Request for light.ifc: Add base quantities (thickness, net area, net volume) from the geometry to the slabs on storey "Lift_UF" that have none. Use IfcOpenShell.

First a look at what the model holds.

```python
import ifcopenshell
import ifcopenshell.util.element
import ifcopenshell.util.unit

model = ifcopenshell.open("light.ifc")
print(model.schema)
for unit_type in ("LENGTHUNIT", "AREAUNIT", "VOLUMEUNIT"):
    print(unit_type, ifcopenshell.util.unit.calculate_unit_scale(model, unit_type))
storey = next(s for s in model.by_type("IfcBuildingStorey") if s.Name == "Lift_UF")
slabs = [e for e in ifcopenshell.util.element.get_decomposition(storey) if e.is_a("IfcSlab")]
for e in sorted(slabs, key=lambda e: e.id()):
    print(e.id(), e.is_a(), e.Name, list(ifcopenshell.util.element.get_psets(e, qtos_only=True)), sep=" | ")
```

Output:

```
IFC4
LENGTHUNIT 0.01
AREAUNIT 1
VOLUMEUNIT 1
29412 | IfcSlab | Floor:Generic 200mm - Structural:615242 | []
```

```python
import ifcopenshell
import ifcopenshell.api.pset
import ifcopenshell.geom
import ifcopenshell.util.element
import ifcopenshell.util.shape
import ifcopenshell.util.unit

model = ifcopenshell.open("light.ifc")
unit_scale = ifcopenshell.util.unit.calculate_unit_scale(model)
area_scale = ifcopenshell.util.unit.calculate_unit_scale(model, "AREAUNIT")
volume_scale = ifcopenshell.util.unit.calculate_unit_scale(model, "VOLUMEUNIT")
settings = ifcopenshell.geom.settings()

storey = next(s for s in model.by_type("IfcBuildingStorey") if s.Name == "Lift_UF")
slabs = [e for e in ifcopenshell.util.element.get_decomposition(storey) if e.is_a("IfcSlab")]

for e in sorted(slabs, key=lambda e: e.id()):
    if ifcopenshell.util.element.get_psets(e, qtos_only=True, should_inherit=False):
        continue
    # Geometry comes back in metres, in the element's own axes.
    shape = ifcopenshell.geom.create_shape(settings, e)
    values = {
        "Width": ifcopenshell.util.shape.get_z(shape.geometry) / unit_scale,
        "NetArea": ifcopenshell.util.shape.get_footprint_area(shape.geometry) / area_scale,
        "NetVolume": ifcopenshell.util.shape.get_volume(shape.geometry) / volume_scale,
    }
    qto = ifcopenshell.api.pset.add_qto(model, product=e, name="Qto_SlabBaseQuantities")
    ifcopenshell.api.pset.edit_qto(model, qto=qto, properties=values)
    print(e.id(), {k: round(v, 3) for k, v in values.items()})

model.write("light_edited.ifc")
```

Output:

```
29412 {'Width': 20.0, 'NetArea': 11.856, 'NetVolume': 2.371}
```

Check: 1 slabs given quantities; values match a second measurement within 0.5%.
